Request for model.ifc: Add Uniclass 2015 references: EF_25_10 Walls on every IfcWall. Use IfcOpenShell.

First a look at what the model holds.

```python
import ifcopenshell

model = ifcopenshell.open("model.ifc")
print(model.schema)
print("classifications:", [c.Name for c in model.by_type("IfcClassification")])
for ifc_class in ("IfcDoor", "IfcRoof", "IfcStair", "IfcWall", "IfcWindow"):
    print(ifc_class, len(model.by_type(ifc_class)))
```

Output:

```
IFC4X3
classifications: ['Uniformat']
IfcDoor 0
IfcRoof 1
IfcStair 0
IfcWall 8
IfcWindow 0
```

```python
import ifcopenshell
import ifcopenshell.api.classification

model = ifcopenshell.open("model.ifc")

system = ifcopenshell.api.classification.add_classification(model, classification="Uniclass 2015")

codes = {
    "IfcWall": ("EF_25_10", "Walls"),
}
for ifc_class, (code, name) in codes.items():
    products = model.by_type(ifc_class)
    ifcopenshell.api.classification.add_reference(
        model, products=products, classification=system, identification=code, name=name
    )
    print(code, len(products))

model.write("model_v2.ifc")
```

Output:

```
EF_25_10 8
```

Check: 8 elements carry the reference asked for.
